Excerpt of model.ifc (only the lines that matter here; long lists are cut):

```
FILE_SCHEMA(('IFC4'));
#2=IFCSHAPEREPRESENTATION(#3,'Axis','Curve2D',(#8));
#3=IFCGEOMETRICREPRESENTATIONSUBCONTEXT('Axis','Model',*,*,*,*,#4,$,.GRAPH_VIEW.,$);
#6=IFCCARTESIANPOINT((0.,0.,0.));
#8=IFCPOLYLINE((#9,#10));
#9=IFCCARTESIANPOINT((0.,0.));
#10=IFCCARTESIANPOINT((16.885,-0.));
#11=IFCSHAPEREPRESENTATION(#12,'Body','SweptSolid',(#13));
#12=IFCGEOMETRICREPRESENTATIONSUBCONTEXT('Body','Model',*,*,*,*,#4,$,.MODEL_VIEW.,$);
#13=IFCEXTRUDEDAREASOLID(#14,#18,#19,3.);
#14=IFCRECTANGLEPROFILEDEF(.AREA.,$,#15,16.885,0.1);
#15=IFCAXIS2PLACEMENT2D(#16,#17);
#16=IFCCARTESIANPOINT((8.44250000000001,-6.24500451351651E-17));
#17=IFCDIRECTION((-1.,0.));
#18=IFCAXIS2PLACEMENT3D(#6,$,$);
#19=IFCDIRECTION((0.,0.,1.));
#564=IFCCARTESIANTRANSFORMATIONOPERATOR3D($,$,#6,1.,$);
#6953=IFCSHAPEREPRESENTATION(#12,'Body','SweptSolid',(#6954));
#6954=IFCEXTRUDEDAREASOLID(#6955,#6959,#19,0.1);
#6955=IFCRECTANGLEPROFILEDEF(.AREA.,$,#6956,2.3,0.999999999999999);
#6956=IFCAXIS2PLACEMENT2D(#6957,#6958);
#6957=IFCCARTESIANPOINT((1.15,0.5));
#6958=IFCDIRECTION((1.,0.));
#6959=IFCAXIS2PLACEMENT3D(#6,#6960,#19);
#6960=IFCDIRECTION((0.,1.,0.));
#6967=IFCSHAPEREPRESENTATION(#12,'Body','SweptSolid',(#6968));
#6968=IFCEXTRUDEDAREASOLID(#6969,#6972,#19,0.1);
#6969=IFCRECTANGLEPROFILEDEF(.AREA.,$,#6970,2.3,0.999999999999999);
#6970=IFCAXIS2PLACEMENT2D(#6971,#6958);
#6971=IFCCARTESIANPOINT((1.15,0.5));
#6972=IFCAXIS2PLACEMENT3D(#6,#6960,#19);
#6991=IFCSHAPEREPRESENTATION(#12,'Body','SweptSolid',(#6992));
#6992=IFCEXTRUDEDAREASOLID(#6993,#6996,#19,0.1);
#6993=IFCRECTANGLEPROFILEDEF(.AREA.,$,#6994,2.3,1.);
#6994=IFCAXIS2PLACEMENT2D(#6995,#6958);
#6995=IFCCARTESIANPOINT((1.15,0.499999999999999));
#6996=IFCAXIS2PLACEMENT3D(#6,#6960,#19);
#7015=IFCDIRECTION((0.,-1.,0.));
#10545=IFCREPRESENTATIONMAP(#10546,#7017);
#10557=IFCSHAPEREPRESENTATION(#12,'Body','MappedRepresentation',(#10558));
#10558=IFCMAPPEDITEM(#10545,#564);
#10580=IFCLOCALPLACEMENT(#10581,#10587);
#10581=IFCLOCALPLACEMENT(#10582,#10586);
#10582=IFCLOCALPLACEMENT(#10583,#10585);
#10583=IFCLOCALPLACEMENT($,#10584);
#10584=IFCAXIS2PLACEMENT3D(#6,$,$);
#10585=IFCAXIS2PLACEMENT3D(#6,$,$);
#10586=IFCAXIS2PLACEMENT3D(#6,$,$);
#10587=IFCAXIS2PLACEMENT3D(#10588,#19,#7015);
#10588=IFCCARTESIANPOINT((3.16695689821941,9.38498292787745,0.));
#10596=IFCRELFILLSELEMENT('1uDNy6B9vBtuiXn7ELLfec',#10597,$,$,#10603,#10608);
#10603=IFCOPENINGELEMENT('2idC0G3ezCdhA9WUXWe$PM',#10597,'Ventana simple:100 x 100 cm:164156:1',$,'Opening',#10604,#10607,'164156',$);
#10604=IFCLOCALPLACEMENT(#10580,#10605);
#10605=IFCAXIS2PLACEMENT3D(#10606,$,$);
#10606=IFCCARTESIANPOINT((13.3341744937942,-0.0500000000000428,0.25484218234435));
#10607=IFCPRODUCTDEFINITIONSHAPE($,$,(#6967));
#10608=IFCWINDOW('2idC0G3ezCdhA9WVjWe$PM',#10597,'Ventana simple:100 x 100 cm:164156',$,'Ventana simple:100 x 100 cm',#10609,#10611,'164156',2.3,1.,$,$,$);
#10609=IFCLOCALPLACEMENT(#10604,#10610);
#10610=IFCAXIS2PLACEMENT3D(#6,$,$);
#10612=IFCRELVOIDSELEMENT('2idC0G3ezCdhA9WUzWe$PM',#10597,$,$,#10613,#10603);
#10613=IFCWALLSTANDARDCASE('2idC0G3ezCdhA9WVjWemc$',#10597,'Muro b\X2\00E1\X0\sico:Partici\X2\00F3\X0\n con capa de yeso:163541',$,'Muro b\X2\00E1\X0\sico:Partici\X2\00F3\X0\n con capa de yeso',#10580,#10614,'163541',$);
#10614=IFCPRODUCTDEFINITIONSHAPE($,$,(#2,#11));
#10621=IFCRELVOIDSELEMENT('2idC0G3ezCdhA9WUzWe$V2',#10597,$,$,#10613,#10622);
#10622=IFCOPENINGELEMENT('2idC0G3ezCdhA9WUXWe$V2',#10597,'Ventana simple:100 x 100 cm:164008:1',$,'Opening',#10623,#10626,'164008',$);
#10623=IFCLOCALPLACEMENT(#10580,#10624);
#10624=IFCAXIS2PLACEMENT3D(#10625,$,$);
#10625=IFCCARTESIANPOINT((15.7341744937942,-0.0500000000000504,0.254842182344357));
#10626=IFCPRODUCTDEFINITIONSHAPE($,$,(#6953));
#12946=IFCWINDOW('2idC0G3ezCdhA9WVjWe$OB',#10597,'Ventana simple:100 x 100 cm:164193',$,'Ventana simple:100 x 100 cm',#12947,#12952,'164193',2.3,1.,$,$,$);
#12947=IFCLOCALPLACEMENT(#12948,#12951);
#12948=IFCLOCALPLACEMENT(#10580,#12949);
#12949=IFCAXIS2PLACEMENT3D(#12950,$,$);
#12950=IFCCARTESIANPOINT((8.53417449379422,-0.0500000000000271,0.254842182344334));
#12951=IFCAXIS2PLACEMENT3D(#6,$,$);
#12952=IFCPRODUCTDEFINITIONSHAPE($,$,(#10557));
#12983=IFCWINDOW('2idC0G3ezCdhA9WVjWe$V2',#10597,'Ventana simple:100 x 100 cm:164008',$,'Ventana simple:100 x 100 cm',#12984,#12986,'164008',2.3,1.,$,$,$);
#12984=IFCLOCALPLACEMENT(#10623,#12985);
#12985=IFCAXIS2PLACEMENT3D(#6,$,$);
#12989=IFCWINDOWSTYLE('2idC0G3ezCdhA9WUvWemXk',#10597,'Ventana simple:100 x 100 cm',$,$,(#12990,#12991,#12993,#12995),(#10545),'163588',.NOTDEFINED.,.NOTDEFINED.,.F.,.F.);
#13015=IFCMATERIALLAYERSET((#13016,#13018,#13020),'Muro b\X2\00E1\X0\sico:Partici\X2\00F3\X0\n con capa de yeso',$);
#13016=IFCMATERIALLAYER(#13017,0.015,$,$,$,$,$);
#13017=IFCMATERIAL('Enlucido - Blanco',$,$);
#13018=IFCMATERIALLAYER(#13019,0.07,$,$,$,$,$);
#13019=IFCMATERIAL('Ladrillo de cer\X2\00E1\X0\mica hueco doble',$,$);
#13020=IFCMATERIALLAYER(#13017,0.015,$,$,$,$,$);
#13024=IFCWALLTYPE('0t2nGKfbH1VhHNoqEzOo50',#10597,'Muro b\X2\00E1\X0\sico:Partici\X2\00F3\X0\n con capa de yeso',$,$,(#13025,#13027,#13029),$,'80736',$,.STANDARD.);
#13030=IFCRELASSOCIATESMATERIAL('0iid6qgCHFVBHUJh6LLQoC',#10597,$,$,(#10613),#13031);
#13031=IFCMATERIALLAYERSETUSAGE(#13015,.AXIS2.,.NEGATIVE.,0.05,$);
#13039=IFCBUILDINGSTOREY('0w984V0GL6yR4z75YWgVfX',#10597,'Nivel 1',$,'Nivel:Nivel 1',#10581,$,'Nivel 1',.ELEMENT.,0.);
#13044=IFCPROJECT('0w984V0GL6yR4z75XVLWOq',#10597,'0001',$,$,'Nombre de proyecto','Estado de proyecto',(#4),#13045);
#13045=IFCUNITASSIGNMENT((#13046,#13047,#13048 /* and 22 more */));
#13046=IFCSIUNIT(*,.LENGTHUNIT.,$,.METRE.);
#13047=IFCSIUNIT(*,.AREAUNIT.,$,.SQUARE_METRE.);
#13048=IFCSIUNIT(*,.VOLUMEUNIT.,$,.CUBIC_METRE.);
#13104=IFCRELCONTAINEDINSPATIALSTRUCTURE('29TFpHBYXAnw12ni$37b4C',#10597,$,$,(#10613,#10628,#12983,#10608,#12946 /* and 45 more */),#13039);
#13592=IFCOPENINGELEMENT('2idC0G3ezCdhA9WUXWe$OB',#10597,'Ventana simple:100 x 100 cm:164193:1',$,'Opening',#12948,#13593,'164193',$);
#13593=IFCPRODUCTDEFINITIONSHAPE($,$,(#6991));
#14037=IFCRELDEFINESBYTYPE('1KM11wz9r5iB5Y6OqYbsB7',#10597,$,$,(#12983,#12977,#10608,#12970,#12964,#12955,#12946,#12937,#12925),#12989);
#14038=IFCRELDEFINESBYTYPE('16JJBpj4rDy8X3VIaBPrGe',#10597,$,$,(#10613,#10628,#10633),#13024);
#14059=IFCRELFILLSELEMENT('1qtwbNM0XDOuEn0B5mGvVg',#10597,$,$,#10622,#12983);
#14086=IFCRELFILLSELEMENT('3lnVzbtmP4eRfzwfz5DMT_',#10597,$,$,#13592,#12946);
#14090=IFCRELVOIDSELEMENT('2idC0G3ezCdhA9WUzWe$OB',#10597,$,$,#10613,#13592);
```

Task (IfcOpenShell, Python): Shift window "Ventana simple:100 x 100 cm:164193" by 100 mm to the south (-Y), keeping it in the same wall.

```python
import ifcopenshell
import ifcopenshell.api.geometry
import ifcopenshell.util.placement

model = ifcopenshell.open("model.ifc")

window = model.by_guid("2idC0G3ezCdhA9WVjWe$OB")
opening = window.FillsVoids[0].RelatingOpeningElement
wall = opening.VoidsElements[0].RelatingBuildingElement

wall_matrix = ifcopenshell.util.placement.get_local_placement(wall.ObjectPlacement)
shift = wall_matrix[:3, 0] * 0.1
before = ifcopenshell.util.placement.get_local_placement(window.ObjectPlacement)[:3, 3].copy()

# The window is placed relative to its opening, so it follows when the opening moves.
matrix = ifcopenshell.util.placement.get_local_placement(opening.ObjectPlacement)
matrix[:3, 3] += shift
ifcopenshell.api.geometry.edit_object_placement(
    model, product=opening, matrix=matrix, is_si=False, should_transform_children=True
)

after = ifcopenshell.util.placement.get_local_placement(window.ObjectPlacement)[:3, 3]
print("window moved by", (after - before).round(3) + 0.0)

model.write("model-out.ifc")
```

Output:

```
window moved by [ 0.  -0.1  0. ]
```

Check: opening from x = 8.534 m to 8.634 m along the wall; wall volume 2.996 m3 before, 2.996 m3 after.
